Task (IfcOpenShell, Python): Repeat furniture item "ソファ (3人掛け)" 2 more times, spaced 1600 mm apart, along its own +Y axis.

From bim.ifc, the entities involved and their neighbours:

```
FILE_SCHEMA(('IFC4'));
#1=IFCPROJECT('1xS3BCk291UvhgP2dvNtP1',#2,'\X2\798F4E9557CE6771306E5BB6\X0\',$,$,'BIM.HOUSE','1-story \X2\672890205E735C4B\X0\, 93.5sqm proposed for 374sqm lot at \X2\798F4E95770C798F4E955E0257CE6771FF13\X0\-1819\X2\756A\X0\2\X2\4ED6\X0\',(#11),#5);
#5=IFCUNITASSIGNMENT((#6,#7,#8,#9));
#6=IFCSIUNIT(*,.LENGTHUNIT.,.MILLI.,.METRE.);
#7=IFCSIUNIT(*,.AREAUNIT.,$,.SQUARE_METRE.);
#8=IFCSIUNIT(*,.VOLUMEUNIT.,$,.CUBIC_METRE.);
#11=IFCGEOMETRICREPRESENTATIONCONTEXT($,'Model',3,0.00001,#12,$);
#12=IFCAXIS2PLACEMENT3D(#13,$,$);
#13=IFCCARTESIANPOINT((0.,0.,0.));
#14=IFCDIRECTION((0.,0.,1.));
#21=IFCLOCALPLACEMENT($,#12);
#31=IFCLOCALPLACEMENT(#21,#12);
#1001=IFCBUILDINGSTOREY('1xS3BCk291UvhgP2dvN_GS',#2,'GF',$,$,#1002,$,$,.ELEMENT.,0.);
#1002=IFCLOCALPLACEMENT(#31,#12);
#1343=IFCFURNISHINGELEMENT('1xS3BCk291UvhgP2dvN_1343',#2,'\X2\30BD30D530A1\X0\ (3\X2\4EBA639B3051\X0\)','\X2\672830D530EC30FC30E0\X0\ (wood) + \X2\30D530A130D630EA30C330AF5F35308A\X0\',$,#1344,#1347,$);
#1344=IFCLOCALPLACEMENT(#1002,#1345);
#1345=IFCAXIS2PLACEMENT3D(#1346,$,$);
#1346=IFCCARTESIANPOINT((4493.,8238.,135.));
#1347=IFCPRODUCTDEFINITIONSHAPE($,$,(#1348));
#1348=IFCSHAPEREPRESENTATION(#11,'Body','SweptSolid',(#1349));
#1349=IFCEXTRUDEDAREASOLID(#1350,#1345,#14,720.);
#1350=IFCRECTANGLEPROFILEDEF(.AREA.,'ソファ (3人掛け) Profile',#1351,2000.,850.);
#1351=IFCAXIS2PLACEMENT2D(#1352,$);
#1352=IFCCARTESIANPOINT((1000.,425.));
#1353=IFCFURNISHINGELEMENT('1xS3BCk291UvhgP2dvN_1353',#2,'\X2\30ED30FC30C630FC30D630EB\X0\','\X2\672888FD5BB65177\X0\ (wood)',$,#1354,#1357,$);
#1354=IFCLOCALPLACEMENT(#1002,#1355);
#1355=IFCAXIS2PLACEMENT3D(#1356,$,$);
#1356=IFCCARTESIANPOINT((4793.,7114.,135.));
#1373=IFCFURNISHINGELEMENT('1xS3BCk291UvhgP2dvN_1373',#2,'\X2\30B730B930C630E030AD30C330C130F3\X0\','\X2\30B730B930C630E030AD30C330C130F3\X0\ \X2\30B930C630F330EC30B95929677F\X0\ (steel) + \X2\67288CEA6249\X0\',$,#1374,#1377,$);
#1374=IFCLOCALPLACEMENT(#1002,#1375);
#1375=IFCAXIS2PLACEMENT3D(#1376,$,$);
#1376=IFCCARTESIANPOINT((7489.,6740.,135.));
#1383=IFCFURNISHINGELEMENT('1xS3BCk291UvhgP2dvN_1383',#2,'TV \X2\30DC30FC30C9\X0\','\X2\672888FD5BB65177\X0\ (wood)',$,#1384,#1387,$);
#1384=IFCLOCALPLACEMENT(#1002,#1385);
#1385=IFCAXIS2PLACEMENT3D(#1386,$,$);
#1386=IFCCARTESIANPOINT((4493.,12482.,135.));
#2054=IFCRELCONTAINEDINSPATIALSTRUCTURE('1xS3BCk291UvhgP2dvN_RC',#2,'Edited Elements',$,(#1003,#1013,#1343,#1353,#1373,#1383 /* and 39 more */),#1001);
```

```python
import ifcopenshell
import ifcopenshell.api.geometry
import ifcopenshell.api.root
import ifcopenshell.util.element
import ifcopenshell.util.placement

model = ifcopenshell.open("bim.ifc")


def reuse_history(source, copy):
    """copy_class also copies each property set's owner history, people and application; keep the originals."""
    for rel in copy.IsDefinedBy:
        if rel.is_a("IfcRelDefinesByProperties") and (history := rel.RelatingPropertyDefinition.OwnerHistory):
            rel.RelatingPropertyDefinition.OwnerHistory = source.OwnerHistory
            ifcopenshell.util.element.remove_deep2(model, history)


source = model.by_guid("1xS3BCk291UvhgP2dvN_1343")
base = ifcopenshell.util.placement.get_local_placement(source.ObjectPlacement)
step = base[:3, 1] * 1600.0

for i in range(1, 3):
    copy = ifcopenshell.api.root.copy_class(model, product=source)
    copy.Representation = ifcopenshell.util.element.copy_deep(
        model, source.Representation, exclude=["IfcGeometricRepresentationContext", "IfcRepresentationMap"]
    )
    reuse_history(source, copy)
    matrix = base.copy()
    matrix[:3, 3] += i * step
    print("added at", matrix[:3, 3].round(3) + 0.0)
    ifcopenshell.api.geometry.edit_object_placement(model, product=copy, matrix=matrix, is_si=False)

model.write("bim_v2.ifc")
```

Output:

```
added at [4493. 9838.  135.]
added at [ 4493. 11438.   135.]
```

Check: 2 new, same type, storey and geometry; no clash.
